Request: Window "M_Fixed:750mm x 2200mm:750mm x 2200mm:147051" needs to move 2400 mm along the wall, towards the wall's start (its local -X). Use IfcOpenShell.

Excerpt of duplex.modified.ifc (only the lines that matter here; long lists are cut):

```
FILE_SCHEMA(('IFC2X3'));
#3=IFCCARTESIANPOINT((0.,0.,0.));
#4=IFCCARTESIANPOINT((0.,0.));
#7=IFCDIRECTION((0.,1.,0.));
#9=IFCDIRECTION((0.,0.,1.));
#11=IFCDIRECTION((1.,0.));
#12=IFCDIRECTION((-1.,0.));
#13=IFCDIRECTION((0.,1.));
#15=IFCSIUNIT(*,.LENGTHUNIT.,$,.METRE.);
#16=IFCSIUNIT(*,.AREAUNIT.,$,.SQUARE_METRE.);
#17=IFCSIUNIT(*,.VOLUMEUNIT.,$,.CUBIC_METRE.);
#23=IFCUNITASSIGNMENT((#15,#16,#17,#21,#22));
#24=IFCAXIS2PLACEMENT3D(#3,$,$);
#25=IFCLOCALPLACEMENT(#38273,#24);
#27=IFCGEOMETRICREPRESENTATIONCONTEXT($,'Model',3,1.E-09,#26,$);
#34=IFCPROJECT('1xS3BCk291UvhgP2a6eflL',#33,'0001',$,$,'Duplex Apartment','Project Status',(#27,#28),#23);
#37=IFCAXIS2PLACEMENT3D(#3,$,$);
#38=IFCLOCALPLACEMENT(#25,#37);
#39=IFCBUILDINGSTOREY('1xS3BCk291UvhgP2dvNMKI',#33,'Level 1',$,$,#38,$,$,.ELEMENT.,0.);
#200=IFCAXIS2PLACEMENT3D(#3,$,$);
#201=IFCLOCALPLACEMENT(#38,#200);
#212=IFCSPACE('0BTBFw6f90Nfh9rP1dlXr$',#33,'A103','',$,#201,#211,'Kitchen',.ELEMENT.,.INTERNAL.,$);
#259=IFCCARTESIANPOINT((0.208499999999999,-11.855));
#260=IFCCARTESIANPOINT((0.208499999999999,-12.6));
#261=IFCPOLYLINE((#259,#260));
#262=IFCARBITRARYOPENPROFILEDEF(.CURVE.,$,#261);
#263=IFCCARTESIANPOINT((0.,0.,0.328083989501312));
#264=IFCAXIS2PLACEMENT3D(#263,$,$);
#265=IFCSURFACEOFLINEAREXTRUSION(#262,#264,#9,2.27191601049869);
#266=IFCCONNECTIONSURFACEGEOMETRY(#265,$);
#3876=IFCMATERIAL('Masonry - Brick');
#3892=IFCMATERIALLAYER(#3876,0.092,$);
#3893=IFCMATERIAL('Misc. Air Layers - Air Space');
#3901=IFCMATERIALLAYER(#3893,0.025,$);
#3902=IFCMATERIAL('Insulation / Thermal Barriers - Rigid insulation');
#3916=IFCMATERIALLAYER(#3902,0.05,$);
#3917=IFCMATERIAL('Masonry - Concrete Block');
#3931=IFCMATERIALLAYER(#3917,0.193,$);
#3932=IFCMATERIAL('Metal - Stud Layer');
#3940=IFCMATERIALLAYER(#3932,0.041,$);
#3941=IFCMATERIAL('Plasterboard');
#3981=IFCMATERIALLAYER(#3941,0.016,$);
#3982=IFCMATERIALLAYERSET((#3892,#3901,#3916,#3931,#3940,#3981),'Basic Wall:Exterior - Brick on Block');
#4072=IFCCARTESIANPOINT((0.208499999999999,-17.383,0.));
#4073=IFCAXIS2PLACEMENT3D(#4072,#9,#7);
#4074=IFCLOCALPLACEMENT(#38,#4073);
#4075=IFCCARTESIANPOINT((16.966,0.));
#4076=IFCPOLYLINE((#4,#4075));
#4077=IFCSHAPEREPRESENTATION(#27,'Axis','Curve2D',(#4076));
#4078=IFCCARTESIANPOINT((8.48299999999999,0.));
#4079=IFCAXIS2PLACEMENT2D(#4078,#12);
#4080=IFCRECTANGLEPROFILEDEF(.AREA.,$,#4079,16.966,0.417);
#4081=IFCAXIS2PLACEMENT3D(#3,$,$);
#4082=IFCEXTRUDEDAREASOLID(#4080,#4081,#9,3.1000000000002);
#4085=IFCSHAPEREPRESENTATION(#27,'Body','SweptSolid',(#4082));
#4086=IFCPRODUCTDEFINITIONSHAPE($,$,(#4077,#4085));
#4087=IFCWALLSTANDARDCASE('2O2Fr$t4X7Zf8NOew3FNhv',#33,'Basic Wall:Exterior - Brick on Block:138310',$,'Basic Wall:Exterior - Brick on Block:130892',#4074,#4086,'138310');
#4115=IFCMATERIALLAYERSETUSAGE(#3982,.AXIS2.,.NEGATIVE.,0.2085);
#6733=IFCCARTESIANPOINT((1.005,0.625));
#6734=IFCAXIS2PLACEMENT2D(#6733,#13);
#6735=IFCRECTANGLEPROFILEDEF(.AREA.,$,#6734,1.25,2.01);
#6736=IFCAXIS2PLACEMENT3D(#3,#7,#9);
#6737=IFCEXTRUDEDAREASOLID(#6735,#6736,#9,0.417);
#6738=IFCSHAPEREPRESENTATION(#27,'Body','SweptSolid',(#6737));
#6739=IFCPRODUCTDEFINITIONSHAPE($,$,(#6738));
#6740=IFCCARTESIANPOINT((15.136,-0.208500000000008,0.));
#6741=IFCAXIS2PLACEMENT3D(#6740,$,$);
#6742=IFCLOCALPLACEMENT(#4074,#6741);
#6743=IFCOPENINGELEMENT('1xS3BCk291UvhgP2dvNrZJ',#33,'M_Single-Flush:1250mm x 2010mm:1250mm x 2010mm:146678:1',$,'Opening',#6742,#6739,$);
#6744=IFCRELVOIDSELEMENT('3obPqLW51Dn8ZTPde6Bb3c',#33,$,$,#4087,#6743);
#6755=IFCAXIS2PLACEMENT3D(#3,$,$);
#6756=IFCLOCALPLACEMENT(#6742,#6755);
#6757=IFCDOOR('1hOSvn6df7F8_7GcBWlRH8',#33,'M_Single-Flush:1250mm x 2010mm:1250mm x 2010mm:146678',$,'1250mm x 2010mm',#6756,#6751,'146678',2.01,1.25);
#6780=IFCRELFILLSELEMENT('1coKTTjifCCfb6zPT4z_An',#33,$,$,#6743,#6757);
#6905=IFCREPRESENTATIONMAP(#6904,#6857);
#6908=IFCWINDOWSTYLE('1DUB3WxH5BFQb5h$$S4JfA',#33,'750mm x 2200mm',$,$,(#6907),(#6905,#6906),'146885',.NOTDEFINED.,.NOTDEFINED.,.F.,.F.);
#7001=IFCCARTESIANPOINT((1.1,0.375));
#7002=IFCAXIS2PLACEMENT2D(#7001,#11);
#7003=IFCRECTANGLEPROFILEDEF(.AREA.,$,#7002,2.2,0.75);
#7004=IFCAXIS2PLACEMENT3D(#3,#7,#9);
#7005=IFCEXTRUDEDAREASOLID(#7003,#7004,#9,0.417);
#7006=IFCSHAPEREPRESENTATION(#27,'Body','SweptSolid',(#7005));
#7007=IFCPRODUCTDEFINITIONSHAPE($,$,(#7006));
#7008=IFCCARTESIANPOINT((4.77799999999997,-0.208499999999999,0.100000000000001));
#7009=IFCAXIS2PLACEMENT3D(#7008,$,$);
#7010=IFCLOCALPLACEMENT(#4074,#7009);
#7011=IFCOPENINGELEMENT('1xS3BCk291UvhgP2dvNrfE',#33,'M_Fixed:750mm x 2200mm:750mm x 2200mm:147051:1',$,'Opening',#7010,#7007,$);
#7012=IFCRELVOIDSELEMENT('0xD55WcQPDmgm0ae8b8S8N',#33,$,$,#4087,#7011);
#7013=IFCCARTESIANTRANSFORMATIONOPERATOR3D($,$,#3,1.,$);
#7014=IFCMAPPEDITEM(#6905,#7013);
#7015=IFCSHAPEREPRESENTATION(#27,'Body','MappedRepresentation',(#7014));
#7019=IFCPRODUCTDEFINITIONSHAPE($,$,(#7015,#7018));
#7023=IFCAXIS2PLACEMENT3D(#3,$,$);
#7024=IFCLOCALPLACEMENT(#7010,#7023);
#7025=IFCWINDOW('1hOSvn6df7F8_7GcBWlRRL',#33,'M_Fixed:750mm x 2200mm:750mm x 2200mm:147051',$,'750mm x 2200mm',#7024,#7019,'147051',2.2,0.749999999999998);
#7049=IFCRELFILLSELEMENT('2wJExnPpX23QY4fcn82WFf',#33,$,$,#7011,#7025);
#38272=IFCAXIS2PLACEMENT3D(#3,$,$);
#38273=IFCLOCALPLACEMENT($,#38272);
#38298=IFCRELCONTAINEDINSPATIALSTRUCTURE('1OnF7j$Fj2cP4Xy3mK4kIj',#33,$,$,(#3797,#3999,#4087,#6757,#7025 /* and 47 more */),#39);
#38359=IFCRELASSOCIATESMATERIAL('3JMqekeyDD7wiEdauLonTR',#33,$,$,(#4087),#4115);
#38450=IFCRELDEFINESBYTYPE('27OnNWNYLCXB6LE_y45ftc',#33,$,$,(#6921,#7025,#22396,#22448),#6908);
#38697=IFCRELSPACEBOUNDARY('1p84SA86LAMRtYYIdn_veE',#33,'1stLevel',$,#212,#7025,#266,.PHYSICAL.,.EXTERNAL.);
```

```python
import numpy as np
import ifcopenshell
import ifcopenshell.api.geometry
import ifcopenshell.util.placement

model = ifcopenshell.open("duplex.modified.ifc")

window = model.by_id(7025)
opening = window.FillsVoids[0].RelatingOpeningElement
wall = opening.VoidsElements[0].RelatingBuildingElement

wall_matrix = ifcopenshell.util.placement.get_local_placement(wall.ObjectPlacement)
shift = wall_matrix[:3, 0] * -2.4
before = ifcopenshell.util.placement.get_local_placement(window.ObjectPlacement)[:3, 3].copy()

# The window is placed relative to its opening, so it follows when the opening moves.
matrix = ifcopenshell.util.placement.get_local_placement(opening.ObjectPlacement)
matrix[:3, 3] += shift
ifcopenshell.api.geometry.edit_object_placement(
    model, product=opening, matrix=matrix, is_si=False, should_transform_children=True
)

# Space boundary surfaces are stored in each space's coordinates; move them too.
for rel in window.ProvidesBoundaries:
    if not rel.ConnectionGeometry:
        continue
    surface = rel.ConnectionGeometry.SurfaceOnRelatingElement
    space_matrix = ifcopenshell.util.placement.get_local_placement(rel.RelatingSpace.ObjectPlacement)
    point = np.array(surface.Position.Location.Coordinates) + space_matrix[:3, :3].T @ shift
    surface.Position = model.createIfcAxis2Placement3D(
        model.createIfcCartesianPoint(point.tolist()), surface.Position.Axis, surface.Position.RefDirection
    )

after = ifcopenshell.util.placement.get_local_placement(window.ObjectPlacement)[:3, 3]
print("window moved by", (after - before).round(3) + 0.0)

model.write("duplex.modified_v2.ifc")
```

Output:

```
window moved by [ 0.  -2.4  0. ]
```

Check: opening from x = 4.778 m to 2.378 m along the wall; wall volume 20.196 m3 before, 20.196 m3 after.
